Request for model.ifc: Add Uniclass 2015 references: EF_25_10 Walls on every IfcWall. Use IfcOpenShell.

First a look at what the model holds.

```python
import ifcopenshell

model = ifcopenshell.open("model.ifc")
print(model.schema)
print("classifications:", [c.Name for c in model.by_type("IfcClassification")])
for ifc_class in ("IfcDoor", "IfcRoof", "IfcStair", "IfcWall", "IfcWindow"):
    print(ifc_class, len(model.by_type(ifc_class)))
```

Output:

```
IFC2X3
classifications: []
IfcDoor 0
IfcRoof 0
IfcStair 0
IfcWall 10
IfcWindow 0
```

```python
import ifcopenshell
import ifcopenshell.api.classification

model = ifcopenshell.open("model.ifc")

# IFC2X3 requires Source and Edition and has no link from the project to the system.
system = model.create_entity("IfcClassification", Source="NBS", Edition="2015", Name="Uniclass 2015")

codes = {
    "IfcWall": ("EF_25_10", "Walls"),
}
for ifc_class, (code, name) in codes.items():
    products = model.by_type(ifc_class)
    ifcopenshell.api.classification.add_reference(
        model, products=products, classification=system, identification=code, name=name
    )
    print(code, len(products))

model.write("model-out.ifc")
```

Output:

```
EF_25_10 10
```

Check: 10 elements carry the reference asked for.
